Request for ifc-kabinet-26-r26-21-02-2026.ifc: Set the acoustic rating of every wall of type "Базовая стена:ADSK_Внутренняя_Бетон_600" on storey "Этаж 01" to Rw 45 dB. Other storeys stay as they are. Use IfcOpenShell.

First a look at what the model holds.

```python
import ifcopenshell
import ifcopenshell.util.element

model = ifcopenshell.open("ifc-kabinet-26-r26-21-02-2026.ifc")
print(model.schema)
storey = next(s for s in model.by_type("IfcBuildingStorey") if s.Name == "Этаж 01")
walls = [e for e in ifcopenshell.util.element.get_decomposition(storey) if e.is_a("IfcWall")]
seen = {}
for e in walls:
    element_type = ifcopenshell.util.element.get_type(e)
    key = (element_type.Name if element_type != e and element_type else None, ifcopenshell.util.element.get_pset(e, "Pset_WallCommon", "AcousticRating"))
    seen[key] = seen.get(key, 0) + 1
for (name, value), count in sorted(seen.items(), key=str):
    print(count, "x", name, "|", value)
```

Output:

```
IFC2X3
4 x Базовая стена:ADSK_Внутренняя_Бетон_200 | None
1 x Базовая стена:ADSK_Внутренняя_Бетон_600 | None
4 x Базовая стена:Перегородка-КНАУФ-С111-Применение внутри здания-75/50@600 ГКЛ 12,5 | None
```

```python
import ifcopenshell
import ifcopenshell.api.pset
import ifcopenshell.util.element

model = ifcopenshell.open("ifc-kabinet-26-r26-21-02-2026.ifc")

storey = next(s for s in model.by_type("IfcBuildingStorey") if s.Name == "Этаж 01")
walls = [e for e in ifcopenshell.util.element.get_decomposition(storey) if e.is_a("IfcWall")]

count = 0
for e in walls:
    element_type = ifcopenshell.util.element.get_type(e)
    if element_type in (None, e) or element_type.Name != "Базовая стена:ADSK_Внутренняя_Бетон_600":
        continue
    # add_pset returns the element's existing set when there is one.
    pset = ifcopenshell.api.pset.add_pset(model, product=e, name="Pset_WallCommon")
    ifcopenshell.api.pset.edit_pset(model, pset=pset, properties={"AcousticRating": "Rw 45 dB"})
    count += 1

print(count, "walls updated")

model.write("ifc-kabinet-26-r26-21-02-2026_rev.ifc")
```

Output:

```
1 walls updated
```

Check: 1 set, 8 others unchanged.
